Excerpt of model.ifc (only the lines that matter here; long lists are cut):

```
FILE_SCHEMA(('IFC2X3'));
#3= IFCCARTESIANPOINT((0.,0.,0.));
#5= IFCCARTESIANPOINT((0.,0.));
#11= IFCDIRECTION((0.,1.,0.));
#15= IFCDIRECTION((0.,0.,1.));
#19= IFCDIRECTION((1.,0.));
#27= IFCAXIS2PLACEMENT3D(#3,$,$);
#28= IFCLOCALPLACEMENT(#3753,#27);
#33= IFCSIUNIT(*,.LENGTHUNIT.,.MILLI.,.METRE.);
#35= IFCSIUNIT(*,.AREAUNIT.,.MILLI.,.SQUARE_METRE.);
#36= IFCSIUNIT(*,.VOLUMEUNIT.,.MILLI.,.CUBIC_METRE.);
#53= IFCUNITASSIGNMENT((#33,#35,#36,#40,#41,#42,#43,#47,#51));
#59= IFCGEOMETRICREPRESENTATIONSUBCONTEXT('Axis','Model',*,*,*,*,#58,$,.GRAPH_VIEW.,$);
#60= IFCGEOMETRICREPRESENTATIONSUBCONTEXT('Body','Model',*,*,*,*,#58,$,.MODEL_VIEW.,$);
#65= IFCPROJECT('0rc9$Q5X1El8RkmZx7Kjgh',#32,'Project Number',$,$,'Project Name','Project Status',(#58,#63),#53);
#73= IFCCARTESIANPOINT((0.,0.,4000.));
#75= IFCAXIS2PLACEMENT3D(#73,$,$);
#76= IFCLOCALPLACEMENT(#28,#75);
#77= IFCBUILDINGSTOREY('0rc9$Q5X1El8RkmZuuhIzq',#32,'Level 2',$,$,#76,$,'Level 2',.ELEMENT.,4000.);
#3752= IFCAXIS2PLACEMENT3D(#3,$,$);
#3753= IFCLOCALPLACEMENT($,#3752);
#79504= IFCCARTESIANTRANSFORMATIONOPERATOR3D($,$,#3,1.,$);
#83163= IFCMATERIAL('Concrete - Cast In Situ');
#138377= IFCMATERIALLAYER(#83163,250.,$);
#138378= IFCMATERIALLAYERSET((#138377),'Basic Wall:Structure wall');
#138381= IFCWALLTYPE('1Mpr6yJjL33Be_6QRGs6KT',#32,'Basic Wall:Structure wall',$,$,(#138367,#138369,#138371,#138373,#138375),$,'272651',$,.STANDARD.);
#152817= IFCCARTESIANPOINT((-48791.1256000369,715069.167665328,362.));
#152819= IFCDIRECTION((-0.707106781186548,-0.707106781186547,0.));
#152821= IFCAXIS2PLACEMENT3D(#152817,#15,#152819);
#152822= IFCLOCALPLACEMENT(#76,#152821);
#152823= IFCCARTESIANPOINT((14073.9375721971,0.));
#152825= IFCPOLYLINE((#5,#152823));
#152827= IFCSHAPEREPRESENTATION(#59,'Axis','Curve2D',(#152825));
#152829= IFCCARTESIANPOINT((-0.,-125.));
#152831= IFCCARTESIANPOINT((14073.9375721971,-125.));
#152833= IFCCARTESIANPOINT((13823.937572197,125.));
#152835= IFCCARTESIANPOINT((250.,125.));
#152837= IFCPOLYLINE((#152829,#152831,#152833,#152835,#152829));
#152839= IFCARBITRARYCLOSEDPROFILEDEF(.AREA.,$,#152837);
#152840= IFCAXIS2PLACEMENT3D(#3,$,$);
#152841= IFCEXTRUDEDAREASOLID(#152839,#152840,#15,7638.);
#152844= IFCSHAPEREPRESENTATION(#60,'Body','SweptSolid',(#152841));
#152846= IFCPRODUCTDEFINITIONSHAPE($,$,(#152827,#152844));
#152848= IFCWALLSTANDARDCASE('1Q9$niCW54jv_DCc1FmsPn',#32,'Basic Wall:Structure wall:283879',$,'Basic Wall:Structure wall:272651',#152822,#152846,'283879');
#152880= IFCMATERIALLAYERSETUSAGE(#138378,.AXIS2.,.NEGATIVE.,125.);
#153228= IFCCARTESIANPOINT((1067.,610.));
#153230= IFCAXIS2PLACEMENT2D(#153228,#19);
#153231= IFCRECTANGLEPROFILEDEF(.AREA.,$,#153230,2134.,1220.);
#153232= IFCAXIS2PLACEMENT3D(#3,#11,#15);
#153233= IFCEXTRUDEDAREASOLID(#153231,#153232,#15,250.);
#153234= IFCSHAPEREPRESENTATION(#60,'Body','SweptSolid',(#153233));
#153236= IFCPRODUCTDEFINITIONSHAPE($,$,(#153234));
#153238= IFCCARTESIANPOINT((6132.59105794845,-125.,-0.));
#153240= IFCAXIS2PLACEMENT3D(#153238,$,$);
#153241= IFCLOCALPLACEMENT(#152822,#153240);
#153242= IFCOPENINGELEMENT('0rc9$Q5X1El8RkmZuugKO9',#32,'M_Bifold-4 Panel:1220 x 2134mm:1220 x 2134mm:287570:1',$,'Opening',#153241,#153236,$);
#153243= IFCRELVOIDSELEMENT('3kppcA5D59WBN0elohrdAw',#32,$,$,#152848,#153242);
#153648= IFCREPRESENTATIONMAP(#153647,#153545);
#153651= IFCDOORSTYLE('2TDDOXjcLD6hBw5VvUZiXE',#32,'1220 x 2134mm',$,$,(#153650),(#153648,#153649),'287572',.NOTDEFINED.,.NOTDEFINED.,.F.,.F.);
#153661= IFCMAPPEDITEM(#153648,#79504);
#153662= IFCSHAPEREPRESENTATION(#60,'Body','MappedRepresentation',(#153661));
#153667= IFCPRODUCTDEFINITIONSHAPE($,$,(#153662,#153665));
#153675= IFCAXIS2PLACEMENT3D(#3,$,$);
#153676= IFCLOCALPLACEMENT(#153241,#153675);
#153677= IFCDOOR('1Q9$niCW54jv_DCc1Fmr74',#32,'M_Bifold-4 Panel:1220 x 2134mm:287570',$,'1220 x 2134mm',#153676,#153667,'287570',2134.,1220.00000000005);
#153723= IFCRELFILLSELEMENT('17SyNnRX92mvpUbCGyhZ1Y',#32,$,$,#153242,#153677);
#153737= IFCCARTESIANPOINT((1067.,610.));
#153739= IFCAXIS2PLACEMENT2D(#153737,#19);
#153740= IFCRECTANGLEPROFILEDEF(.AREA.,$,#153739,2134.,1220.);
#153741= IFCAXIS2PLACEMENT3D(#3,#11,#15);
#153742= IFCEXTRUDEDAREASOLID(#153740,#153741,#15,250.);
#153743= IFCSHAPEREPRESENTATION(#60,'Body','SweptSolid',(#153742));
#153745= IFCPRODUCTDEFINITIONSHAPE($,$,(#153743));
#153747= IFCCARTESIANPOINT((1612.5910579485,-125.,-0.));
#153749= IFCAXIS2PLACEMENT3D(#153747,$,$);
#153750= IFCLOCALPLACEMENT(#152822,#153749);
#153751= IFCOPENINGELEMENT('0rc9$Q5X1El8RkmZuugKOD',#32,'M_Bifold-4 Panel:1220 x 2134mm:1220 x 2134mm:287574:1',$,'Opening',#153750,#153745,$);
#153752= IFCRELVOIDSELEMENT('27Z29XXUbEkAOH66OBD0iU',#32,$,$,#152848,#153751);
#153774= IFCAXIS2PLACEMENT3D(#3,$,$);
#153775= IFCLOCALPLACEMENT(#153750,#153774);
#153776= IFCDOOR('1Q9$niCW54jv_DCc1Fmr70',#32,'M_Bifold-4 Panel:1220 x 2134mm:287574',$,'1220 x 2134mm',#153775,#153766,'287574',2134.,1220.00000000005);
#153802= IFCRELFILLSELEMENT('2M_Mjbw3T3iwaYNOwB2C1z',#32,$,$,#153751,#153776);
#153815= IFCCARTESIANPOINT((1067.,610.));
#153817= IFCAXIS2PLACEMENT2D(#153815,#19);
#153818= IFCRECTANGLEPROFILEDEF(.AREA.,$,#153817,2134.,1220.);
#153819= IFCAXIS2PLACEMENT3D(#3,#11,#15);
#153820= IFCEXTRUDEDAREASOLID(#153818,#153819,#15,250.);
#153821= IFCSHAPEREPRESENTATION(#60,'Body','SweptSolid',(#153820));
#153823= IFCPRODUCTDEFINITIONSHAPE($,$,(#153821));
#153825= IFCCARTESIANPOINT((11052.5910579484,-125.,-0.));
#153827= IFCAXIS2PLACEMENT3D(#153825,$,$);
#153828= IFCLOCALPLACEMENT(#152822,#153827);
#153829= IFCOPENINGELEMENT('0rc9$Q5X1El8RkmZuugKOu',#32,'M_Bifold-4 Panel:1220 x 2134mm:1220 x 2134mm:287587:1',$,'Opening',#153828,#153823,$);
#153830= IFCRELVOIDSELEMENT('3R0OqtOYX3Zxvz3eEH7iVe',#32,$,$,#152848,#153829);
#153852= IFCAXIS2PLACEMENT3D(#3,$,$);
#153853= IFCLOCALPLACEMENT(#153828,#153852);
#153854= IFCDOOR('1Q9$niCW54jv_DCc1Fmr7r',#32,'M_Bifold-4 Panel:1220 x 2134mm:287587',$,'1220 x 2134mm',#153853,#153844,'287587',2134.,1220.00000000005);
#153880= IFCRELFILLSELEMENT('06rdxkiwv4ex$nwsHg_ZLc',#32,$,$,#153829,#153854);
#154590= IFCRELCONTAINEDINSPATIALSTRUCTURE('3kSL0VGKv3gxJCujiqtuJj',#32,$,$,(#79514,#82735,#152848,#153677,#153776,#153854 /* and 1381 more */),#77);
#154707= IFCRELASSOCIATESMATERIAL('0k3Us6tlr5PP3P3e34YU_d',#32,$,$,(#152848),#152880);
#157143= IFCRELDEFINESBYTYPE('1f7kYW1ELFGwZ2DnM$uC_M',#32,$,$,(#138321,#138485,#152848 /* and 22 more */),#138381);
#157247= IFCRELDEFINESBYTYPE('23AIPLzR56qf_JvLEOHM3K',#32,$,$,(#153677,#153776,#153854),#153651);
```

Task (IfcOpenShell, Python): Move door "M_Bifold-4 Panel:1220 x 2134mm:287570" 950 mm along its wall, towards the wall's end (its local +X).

```python
import ifcopenshell
import ifcopenshell.api.geometry
import ifcopenshell.util.placement
import ifcopenshell.util.unit

model = ifcopenshell.open("model.ifc")
unit_scale = ifcopenshell.util.unit.calculate_unit_scale(model)

door = model.by_guid("1Q9$niCW54jv_DCc1Fmr74")
opening = door.FillsVoids[0].RelatingOpeningElement
wall = opening.VoidsElements[0].RelatingBuildingElement

wall_matrix = ifcopenshell.util.placement.get_local_placement(wall.ObjectPlacement)
shift = wall_matrix[:3, 0] * 0.95 / unit_scale
before = ifcopenshell.util.placement.get_local_placement(door.ObjectPlacement)[:3, 3].copy()

# The door is placed relative to its opening, so it follows when the opening moves.
matrix = ifcopenshell.util.placement.get_local_placement(opening.ObjectPlacement)
matrix[:3, 3] += shift
ifcopenshell.api.geometry.edit_object_placement(
    model, product=opening, matrix=matrix, is_si=False, should_transform_children=True
)

after = ifcopenshell.util.placement.get_local_placement(door.ObjectPlacement)[:3, 3]
print("door moved by", (after - before).round(3) + 0.0)

model.write("model-out.ifc")
```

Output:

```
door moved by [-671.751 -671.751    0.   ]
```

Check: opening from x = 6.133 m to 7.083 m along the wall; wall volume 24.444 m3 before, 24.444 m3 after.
